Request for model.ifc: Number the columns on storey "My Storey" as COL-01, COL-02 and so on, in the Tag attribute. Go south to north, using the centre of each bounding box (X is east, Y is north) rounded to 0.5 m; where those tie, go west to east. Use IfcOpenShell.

First a look at what the model holds.

```python
import ifcopenshell
import ifcopenshell.util.element
import ifcopenshell.util.placement

model = ifcopenshell.open("model.ifc")
print(model.schema)
storey = next(s for s in model.by_type("IfcBuildingStorey") if s.Name == "My Storey")
columns = [e for e in ifcopenshell.util.element.get_decomposition(storey) if e.is_a("IfcColumn")]
for e in sorted(columns, key=lambda e: e.id()):
    origin = ifcopenshell.util.placement.get_local_placement(e.ObjectPlacement)[:3, 3]
    print(e.id(), e.Tag, e.Name, origin.round(2) + 0.0, sep=" | ")
```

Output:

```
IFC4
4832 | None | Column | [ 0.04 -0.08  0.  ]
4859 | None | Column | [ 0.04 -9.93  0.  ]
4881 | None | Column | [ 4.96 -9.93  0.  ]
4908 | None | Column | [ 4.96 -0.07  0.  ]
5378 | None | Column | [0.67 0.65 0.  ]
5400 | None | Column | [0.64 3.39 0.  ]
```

```python
import ifcopenshell
import ifcopenshell.geom
import ifcopenshell.util.element
import ifcopenshell.util.shape

model = ifcopenshell.open("model.ifc")
settings = ifcopenshell.geom.settings()
settings.set("use-world-coords", True)


def centre(element):
    shape = ifcopenshell.geom.create_shape(settings, element)
    return ifcopenshell.util.shape.get_bbox_centroid(shape.geometry)


storey = next(s for s in model.by_type("IfcBuildingStorey") if s.Name == "My Storey")
columns = [e for e in ifcopenshell.util.element.get_decomposition(storey) if e.is_a("IfcColumn")]

# Insertion points can sit at a corner or the storey origin, so sort by the geometry (in metres).
centres = {e: centre(e) for e in columns}
columns.sort(key=lambda e: (round(centres[e][1] / 0.5), centres[e][0]))

for i, e in enumerate(columns, start=1):
    number = f"COL-{i:02d}"
    e.Tag = number
    print(e.id(), number)

model.write("model_edited.ifc")
```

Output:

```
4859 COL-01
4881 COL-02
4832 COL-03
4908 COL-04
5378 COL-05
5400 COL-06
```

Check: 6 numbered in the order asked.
